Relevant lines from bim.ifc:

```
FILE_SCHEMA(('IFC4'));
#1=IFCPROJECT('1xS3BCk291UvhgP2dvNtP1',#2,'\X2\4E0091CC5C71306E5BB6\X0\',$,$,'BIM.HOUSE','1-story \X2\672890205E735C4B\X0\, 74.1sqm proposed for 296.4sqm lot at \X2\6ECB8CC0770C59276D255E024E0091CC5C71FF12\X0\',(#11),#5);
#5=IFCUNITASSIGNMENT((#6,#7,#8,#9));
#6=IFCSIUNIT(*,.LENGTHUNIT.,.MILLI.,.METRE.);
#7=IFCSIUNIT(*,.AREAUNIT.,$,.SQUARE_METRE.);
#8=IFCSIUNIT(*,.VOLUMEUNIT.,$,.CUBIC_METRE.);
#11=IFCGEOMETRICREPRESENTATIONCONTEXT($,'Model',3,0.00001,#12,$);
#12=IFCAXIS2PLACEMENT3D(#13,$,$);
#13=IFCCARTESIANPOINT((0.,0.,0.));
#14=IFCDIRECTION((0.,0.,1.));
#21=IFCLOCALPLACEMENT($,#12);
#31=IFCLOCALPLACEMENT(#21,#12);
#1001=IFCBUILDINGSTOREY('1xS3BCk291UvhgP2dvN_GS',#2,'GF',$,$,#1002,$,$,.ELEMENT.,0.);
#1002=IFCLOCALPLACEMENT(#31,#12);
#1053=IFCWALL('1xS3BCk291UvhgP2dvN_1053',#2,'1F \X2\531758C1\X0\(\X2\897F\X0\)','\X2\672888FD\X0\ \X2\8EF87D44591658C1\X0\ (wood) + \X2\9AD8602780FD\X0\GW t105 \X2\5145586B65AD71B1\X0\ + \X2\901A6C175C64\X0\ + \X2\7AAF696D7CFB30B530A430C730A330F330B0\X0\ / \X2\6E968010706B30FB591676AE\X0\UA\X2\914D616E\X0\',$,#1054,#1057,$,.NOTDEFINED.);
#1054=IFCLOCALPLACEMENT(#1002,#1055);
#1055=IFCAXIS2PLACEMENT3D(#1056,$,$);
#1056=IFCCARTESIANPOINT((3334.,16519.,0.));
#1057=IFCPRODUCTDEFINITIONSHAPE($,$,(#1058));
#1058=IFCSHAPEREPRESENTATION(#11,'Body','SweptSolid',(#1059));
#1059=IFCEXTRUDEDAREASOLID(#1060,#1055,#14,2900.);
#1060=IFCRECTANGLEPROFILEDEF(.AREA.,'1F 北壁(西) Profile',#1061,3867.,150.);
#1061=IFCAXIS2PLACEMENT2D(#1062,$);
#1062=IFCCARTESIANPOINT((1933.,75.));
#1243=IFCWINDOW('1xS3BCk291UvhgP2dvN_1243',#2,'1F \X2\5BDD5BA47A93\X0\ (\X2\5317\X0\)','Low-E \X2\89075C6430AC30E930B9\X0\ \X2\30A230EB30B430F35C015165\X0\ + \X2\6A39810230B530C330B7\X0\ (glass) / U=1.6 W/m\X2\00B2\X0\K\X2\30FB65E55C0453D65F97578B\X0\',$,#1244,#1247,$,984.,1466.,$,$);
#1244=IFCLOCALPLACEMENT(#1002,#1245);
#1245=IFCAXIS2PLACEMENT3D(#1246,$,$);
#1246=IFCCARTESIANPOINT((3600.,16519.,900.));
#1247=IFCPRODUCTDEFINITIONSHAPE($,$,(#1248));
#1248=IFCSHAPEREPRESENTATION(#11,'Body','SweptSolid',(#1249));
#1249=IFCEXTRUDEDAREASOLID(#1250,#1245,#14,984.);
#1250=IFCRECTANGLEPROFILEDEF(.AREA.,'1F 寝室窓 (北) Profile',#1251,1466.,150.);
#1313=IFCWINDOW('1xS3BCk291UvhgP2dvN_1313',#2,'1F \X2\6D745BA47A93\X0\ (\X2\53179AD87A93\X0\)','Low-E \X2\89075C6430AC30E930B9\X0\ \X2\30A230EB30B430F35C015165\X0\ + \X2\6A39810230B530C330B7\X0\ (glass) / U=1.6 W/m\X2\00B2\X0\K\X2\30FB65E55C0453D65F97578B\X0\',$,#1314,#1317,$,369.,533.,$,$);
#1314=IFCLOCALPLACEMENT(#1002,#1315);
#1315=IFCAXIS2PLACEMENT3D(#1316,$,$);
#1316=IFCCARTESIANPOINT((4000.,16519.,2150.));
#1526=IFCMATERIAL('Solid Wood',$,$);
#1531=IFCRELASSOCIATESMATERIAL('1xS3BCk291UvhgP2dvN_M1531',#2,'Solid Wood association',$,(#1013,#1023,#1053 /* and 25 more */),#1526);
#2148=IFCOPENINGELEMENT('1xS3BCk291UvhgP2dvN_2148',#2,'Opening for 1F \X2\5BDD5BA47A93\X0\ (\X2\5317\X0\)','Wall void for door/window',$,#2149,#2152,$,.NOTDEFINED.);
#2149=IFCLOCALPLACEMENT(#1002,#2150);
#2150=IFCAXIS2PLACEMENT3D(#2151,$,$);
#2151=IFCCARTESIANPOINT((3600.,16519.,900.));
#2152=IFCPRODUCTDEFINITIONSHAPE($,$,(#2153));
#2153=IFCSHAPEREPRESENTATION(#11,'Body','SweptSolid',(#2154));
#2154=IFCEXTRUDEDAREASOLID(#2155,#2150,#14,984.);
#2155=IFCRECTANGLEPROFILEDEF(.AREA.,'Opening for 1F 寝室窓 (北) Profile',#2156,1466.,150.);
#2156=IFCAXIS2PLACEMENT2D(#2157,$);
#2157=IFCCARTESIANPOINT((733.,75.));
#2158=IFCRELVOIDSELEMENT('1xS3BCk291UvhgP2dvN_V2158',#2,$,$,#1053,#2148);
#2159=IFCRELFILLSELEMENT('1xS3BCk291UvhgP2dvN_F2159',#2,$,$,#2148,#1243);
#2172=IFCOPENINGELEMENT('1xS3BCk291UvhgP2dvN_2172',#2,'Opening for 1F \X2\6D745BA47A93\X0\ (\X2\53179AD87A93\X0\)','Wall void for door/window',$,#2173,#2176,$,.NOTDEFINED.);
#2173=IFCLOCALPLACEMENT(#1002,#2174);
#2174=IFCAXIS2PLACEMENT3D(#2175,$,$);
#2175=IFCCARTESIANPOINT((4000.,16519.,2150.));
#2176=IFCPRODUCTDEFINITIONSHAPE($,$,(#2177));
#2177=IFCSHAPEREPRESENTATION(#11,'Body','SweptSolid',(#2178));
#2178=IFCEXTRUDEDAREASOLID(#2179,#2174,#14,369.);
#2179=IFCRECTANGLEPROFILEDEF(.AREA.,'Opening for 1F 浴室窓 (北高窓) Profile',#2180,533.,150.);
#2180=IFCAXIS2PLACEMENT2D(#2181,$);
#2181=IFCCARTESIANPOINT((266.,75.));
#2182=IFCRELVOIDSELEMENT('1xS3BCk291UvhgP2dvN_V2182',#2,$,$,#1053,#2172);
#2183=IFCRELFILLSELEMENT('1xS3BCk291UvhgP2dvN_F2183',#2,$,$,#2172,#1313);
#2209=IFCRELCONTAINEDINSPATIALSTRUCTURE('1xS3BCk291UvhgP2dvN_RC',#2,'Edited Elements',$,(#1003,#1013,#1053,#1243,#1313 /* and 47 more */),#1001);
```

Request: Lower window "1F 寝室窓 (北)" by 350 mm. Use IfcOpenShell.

```python
import numpy as np
import ifcopenshell
import ifcopenshell.api.geometry
import ifcopenshell.util.placement
import ifcopenshell.util.unit

model = ifcopenshell.open("bim.ifc")
unit_scale = ifcopenshell.util.unit.calculate_unit_scale(model)

window = model.by_guid("1xS3BCk291UvhgP2dvN_1243")
opening = window.FillsVoids[0].RelatingOpeningElement
dz = -350.0

shift = np.array([0.0, 0.0, dz])
# The window is not placed relative to its opening, so move both.
for product in (opening, window):
    matrix = ifcopenshell.util.placement.get_local_placement(product.ObjectPlacement)
    matrix[:3, 3] += shift
    ifcopenshell.api.geometry.edit_object_placement(model, product=product, matrix=matrix, is_si=False)

print(f"moved by {dz * unit_scale:+.3f} m")

model.write("bim_updated.ifc")
```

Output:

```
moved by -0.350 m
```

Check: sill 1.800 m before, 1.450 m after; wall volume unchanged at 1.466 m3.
